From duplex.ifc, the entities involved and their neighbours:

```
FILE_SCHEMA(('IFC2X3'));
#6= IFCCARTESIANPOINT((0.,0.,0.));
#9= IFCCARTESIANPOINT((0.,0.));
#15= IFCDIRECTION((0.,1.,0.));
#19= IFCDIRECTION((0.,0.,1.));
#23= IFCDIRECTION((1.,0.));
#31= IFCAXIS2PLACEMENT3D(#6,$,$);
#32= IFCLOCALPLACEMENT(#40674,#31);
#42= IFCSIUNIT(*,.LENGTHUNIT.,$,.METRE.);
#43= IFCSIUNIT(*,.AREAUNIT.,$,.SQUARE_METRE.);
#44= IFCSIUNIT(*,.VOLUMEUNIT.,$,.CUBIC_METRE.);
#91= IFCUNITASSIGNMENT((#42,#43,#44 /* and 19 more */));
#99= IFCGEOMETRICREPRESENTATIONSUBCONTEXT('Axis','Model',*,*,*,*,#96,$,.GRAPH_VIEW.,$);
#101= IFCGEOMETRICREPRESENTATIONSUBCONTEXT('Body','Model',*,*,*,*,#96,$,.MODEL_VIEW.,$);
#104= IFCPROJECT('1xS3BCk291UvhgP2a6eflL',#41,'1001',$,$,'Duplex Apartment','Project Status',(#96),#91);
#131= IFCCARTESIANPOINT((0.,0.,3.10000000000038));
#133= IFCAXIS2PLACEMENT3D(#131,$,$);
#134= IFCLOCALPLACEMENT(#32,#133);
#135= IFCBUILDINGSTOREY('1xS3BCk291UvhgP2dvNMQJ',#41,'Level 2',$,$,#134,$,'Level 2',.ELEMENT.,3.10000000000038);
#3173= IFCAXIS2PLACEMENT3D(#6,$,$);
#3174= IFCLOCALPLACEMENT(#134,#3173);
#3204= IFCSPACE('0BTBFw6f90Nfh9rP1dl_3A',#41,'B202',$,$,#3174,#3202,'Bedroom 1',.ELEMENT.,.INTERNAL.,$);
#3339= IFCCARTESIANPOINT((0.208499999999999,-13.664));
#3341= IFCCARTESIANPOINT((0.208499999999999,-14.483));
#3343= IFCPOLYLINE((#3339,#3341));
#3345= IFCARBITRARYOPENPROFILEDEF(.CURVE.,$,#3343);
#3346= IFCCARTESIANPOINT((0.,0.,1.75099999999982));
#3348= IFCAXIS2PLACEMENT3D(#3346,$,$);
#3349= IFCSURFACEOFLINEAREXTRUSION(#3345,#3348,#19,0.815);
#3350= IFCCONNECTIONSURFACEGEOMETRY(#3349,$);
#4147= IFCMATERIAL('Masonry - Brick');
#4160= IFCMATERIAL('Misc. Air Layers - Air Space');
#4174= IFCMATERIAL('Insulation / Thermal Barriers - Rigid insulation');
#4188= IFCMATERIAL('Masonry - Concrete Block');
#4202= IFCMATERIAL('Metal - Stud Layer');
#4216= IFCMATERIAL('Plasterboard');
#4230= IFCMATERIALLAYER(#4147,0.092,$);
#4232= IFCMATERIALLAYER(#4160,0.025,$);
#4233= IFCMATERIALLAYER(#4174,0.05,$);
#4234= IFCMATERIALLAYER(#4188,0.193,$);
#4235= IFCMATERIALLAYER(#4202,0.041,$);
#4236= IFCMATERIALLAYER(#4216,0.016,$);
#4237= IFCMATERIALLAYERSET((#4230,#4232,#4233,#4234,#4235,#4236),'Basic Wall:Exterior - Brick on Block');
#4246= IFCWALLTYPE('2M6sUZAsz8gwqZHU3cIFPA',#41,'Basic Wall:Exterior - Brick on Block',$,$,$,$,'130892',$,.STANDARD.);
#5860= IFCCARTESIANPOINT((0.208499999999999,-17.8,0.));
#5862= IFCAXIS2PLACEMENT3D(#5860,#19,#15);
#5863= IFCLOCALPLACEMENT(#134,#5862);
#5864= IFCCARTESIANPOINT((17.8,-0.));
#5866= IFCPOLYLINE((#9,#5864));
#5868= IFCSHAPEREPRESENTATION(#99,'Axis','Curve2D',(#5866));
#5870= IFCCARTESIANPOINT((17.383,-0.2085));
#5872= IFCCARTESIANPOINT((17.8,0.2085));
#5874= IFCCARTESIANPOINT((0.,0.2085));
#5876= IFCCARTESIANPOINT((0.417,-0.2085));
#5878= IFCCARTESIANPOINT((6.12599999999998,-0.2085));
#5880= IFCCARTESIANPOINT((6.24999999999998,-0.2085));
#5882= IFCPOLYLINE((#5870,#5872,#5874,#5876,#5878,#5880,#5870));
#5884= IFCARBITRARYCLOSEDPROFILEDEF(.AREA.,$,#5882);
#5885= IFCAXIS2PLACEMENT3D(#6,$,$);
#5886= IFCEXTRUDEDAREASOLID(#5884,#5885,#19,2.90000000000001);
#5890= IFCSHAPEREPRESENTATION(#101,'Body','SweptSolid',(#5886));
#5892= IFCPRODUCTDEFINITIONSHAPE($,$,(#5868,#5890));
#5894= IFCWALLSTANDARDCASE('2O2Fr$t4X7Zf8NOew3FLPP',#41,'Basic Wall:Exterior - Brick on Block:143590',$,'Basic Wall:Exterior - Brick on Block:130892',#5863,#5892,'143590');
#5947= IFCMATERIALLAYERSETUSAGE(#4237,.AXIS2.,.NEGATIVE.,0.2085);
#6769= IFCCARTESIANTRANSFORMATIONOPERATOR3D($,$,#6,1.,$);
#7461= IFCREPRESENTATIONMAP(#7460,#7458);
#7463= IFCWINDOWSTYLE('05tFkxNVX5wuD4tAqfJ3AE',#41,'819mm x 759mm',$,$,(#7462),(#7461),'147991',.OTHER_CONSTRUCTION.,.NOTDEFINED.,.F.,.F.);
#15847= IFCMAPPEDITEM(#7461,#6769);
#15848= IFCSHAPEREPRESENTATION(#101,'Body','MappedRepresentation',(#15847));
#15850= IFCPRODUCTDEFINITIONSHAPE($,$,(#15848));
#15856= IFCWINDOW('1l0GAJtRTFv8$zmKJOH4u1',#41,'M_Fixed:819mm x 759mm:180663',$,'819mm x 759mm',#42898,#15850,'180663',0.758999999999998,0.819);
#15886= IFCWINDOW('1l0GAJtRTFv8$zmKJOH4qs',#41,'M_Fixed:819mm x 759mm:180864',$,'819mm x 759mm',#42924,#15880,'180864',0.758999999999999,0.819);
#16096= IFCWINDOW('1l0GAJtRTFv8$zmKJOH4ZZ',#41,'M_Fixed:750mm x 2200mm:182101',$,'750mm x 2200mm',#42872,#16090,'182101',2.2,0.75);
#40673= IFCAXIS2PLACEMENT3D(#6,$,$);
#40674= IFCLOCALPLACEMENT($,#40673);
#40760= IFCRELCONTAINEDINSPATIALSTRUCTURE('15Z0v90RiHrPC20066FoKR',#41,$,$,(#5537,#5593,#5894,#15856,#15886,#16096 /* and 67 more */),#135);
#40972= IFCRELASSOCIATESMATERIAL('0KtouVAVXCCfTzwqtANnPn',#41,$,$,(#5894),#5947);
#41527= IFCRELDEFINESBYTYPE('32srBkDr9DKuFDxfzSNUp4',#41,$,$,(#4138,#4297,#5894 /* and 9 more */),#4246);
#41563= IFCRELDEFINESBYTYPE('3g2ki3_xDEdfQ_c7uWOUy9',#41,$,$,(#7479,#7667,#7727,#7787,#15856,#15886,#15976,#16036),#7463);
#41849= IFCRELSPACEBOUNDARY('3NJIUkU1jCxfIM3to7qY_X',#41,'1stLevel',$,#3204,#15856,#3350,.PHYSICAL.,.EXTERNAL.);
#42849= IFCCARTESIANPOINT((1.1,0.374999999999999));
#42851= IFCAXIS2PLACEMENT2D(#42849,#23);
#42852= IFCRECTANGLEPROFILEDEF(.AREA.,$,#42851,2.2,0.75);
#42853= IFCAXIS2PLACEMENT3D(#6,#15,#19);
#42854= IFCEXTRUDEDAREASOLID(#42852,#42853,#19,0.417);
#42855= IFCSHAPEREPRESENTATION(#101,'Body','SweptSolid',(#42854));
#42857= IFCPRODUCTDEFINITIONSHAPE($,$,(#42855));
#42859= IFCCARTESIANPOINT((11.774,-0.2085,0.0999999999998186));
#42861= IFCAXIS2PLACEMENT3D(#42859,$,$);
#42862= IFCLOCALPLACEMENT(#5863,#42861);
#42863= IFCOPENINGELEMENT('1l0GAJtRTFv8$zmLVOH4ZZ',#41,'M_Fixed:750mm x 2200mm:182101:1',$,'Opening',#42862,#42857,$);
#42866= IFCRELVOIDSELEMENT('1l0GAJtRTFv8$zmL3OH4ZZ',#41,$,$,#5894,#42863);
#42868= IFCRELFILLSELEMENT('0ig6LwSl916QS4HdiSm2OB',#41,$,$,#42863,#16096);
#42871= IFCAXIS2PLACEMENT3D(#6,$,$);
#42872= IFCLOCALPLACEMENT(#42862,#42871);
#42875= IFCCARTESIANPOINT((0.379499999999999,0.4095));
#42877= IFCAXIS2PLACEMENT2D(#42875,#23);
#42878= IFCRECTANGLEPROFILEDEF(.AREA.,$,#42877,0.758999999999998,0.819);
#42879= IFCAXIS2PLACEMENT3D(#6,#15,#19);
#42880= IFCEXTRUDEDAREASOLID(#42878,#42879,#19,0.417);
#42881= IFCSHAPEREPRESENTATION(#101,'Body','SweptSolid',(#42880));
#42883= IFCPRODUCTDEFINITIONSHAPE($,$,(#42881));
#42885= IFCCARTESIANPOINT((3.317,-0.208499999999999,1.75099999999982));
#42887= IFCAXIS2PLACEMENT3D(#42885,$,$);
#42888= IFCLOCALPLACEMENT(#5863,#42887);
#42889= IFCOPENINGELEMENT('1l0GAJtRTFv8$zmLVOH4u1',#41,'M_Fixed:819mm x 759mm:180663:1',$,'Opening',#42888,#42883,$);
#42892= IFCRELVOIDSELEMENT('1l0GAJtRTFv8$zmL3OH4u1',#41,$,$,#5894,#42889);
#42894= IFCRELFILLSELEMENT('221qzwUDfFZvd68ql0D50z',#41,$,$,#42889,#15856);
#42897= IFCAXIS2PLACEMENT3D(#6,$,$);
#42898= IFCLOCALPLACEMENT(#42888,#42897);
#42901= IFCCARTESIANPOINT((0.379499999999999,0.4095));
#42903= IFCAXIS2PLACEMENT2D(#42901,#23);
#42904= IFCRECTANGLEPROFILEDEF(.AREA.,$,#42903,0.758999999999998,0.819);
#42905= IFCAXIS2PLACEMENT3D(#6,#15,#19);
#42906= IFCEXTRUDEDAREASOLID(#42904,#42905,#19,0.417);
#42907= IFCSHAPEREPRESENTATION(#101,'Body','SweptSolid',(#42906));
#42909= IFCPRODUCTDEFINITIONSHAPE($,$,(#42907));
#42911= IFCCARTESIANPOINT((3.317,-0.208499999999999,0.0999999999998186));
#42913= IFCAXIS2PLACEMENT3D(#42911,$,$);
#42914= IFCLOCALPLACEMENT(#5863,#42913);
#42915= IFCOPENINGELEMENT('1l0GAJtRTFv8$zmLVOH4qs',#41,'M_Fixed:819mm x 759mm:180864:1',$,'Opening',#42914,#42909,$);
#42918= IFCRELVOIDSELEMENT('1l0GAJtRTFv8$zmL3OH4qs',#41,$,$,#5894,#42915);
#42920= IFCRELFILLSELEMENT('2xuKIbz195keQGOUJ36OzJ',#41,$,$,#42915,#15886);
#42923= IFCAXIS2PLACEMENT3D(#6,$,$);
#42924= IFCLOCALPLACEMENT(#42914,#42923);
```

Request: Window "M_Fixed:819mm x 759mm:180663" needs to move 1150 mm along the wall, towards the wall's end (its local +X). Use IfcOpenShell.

```python
import numpy as np
import ifcopenshell
import ifcopenshell.api.geometry
import ifcopenshell.util.placement

model = ifcopenshell.open("duplex.ifc")

window = model.by_id(15856)
opening = window.FillsVoids[0].RelatingOpeningElement
wall = opening.VoidsElements[0].RelatingBuildingElement

wall_matrix = ifcopenshell.util.placement.get_local_placement(wall.ObjectPlacement)
shift = wall_matrix[:3, 0] * 1.15
before = ifcopenshell.util.placement.get_local_placement(window.ObjectPlacement)[:3, 3].copy()

# The window is placed relative to its opening, so it follows when the opening moves.
matrix = ifcopenshell.util.placement.get_local_placement(opening.ObjectPlacement)
matrix[:3, 3] += shift
ifcopenshell.api.geometry.edit_object_placement(
    model, product=opening, matrix=matrix, is_si=False, should_transform_children=True
)

# Space boundary surfaces are stored in each space's coordinates; move them too.
for rel in window.ProvidesBoundaries:
    if not rel.ConnectionGeometry:
        continue
    surface = rel.ConnectionGeometry.SurfaceOnRelatingElement
    space_matrix = ifcopenshell.util.placement.get_local_placement(rel.RelatingSpace.ObjectPlacement)
    point = np.array(surface.Position.Location.Coordinates) + space_matrix[:3, :3].T @ shift
    surface.Position = model.createIfcAxis2Placement3D(
        model.createIfcCartesianPoint(point.tolist()), surface.Position.Axis, surface.Position.RefDirection
    )

after = ifcopenshell.util.placement.get_local_placement(window.ObjectPlacement)[:3, 3]
print("window moved by", (after - before).round(3) + 0.0)

model.write("duplex-out.ifc")
```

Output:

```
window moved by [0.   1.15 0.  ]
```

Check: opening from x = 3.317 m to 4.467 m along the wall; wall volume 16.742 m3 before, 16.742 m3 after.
